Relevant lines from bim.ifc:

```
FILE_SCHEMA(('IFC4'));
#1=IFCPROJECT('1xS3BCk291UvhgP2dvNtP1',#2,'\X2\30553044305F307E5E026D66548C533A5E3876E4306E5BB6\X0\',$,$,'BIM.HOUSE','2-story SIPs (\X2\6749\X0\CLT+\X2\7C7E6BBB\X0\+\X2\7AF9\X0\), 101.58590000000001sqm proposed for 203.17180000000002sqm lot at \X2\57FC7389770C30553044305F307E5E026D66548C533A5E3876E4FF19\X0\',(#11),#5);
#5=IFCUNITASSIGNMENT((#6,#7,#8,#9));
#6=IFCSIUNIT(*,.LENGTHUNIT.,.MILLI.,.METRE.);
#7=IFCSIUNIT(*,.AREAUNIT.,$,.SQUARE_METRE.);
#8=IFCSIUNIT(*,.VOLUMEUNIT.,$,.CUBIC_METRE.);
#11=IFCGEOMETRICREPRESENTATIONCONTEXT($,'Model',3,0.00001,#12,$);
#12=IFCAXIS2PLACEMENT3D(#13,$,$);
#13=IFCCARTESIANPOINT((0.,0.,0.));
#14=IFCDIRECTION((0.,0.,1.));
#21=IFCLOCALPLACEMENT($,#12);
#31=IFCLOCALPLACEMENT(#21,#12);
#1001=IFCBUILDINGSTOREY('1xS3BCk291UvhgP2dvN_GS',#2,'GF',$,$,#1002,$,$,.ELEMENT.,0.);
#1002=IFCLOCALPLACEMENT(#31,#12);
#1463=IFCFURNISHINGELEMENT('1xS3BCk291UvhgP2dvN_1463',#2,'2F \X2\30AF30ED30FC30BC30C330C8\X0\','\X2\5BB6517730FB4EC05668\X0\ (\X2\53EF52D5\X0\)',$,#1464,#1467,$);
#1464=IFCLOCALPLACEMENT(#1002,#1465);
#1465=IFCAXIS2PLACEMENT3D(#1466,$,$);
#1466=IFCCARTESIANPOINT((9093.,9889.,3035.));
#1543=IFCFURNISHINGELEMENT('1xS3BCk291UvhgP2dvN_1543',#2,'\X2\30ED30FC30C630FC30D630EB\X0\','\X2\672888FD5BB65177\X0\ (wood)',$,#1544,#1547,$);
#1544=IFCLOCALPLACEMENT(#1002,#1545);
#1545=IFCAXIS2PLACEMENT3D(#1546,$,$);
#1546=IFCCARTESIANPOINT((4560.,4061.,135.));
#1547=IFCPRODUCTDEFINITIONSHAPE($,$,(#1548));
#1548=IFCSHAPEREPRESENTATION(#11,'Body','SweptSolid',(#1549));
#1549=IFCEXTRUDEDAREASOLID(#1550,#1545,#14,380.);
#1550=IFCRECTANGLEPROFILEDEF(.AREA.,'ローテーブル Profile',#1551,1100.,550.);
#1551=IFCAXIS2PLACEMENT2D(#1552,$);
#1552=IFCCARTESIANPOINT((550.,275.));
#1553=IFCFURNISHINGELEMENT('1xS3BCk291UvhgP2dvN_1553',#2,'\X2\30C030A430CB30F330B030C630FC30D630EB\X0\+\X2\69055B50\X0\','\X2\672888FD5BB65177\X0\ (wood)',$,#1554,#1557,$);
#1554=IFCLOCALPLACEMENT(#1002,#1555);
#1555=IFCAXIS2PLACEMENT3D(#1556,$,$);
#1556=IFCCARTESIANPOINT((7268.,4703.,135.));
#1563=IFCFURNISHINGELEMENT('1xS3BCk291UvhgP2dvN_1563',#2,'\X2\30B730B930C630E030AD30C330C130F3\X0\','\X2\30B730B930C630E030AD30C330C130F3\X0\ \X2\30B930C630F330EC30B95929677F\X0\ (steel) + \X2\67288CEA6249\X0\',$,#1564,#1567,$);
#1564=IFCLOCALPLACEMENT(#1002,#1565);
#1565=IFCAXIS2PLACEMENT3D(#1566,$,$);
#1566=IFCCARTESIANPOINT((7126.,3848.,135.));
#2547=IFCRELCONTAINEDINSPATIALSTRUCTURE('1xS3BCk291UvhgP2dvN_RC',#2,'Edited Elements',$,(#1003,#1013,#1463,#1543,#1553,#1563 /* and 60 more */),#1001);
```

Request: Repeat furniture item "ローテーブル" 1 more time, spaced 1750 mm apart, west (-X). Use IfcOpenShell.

```python
import numpy as np
import ifcopenshell
import ifcopenshell.api.geometry
import ifcopenshell.api.root
import ifcopenshell.util.element
import ifcopenshell.util.placement
import ifcopenshell.util.unit

model = ifcopenshell.open("bim.ifc")
unit_scale = ifcopenshell.util.unit.calculate_unit_scale(model)


def reuse_history(source, copy):
    """copy_class also copies each property set's owner history, people and application; keep the originals."""
    for rel in copy.IsDefinedBy:
        if rel.is_a("IfcRelDefinesByProperties") and (history := rel.RelatingPropertyDefinition.OwnerHistory):
            rel.RelatingPropertyDefinition.OwnerHistory = source.OwnerHistory
            ifcopenshell.util.element.remove_deep2(model, history)


source = model.by_guid("1xS3BCk291UvhgP2dvN_1543")
base = ifcopenshell.util.placement.get_local_placement(source.ObjectPlacement)
step = np.array([-1.0, 0.0, 0.0]) * 1.75 / unit_scale

for i in range(1, 2):
    copy = ifcopenshell.api.root.copy_class(model, product=source)
    copy.Representation = ifcopenshell.util.element.copy_deep(
        model, source.Representation, exclude=["IfcGeometricRepresentationContext", "IfcRepresentationMap"]
    )
    reuse_history(source, copy)
    matrix = base.copy()
    matrix[:3, 3] += i * step
    print("added at", matrix[:3, 3].round(3) + 0.0)
    ifcopenshell.api.geometry.edit_object_placement(model, product=copy, matrix=matrix, is_si=False)

model.write("bim-out.ifc")
```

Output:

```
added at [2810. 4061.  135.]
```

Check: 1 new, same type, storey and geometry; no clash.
